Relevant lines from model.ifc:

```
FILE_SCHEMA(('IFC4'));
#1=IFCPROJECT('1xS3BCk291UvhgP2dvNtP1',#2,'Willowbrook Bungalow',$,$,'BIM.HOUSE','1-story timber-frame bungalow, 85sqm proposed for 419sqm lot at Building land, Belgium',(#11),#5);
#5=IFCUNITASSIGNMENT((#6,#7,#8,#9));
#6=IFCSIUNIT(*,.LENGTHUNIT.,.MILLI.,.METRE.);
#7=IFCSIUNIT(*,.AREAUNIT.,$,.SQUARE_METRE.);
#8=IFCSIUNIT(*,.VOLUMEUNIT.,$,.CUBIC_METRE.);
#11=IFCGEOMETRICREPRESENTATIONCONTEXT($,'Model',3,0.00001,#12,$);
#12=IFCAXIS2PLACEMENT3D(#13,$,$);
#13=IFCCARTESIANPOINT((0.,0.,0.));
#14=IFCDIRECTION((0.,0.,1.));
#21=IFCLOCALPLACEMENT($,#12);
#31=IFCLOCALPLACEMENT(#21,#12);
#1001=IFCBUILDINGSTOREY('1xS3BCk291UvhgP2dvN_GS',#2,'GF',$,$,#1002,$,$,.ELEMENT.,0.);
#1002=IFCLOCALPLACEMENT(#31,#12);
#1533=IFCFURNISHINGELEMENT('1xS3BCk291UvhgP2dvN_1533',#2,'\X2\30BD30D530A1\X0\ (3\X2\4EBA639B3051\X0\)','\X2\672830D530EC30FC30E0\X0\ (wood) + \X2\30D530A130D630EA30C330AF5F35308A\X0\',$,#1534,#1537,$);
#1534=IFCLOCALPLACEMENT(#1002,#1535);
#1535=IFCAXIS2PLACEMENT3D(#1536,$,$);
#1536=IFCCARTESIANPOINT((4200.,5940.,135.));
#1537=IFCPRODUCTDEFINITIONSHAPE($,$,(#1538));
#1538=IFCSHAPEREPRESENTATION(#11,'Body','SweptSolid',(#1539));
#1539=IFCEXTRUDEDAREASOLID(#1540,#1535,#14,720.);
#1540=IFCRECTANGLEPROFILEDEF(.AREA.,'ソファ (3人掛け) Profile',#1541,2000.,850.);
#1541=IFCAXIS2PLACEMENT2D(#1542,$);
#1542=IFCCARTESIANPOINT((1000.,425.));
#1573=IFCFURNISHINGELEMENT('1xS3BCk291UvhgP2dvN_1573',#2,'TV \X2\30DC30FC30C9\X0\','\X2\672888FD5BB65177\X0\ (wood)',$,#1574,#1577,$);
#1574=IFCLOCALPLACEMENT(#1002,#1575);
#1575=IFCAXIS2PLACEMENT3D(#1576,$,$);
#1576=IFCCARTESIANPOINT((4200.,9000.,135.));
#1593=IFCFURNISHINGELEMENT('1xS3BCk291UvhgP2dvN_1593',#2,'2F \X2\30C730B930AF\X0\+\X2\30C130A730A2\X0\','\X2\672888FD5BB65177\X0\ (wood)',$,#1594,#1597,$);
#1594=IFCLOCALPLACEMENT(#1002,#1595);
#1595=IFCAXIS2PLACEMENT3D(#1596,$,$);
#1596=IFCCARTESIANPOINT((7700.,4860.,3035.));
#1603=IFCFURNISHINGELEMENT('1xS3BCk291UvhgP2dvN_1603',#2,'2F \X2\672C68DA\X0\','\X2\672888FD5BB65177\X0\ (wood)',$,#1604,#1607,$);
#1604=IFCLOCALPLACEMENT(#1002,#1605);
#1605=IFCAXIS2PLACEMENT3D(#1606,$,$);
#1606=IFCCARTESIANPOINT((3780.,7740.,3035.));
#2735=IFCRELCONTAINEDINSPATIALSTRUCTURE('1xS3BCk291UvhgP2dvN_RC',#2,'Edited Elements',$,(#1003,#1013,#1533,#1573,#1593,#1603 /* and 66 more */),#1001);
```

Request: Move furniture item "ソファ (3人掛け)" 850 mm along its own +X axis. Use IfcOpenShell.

```python
import ifcopenshell
import ifcopenshell.api.geometry
import ifcopenshell.util.placement

model = ifcopenshell.open("model.ifc")

item = model.by_guid("1xS3BCk291UvhgP2dvN_1533")
matrix = ifcopenshell.util.placement.get_local_placement(item.ObjectPlacement)
matrix[:3, 3] += matrix[:3, 0] * 850.0
ifcopenshell.api.geometry.edit_object_placement(model, product=item, matrix=matrix, is_si=False)

print(ifcopenshell.util.placement.get_local_placement(item.ObjectPlacement).round(3) + 0.0)

model.write("model_rev.ifc")
```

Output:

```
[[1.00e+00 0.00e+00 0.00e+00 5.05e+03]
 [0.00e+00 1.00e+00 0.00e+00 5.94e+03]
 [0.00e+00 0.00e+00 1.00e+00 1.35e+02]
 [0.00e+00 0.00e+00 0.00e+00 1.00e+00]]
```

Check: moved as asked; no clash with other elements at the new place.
